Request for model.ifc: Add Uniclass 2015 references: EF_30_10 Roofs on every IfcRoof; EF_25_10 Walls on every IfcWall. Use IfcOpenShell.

First a look at what the model holds.

```python
import ifcopenshell

model = ifcopenshell.open("model.ifc")
print(model.schema)
print("classifications:", [c.Name for c in model.by_type("IfcClassification")])
for ifc_class in ("IfcDoor", "IfcRoof", "IfcStair", "IfcWall", "IfcWindow"):
    print(ifc_class, len(model.by_type(ifc_class)))
```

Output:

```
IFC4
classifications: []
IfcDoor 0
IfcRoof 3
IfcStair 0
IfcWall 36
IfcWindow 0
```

```python
import ifcopenshell
import ifcopenshell.api.classification

model = ifcopenshell.open("model.ifc")

system = ifcopenshell.api.classification.add_classification(model, classification="Uniclass 2015")

codes = {
    "IfcRoof": ("EF_30_10", "Roofs"),
    "IfcWall": ("EF_25_10", "Walls"),
}
for ifc_class, (code, name) in codes.items():
    products = model.by_type(ifc_class)
    ifcopenshell.api.classification.add_reference(
        model, products=products, classification=system, identification=code, name=name
    )
    print(code, len(products))

model.write("model_rev.ifc")
```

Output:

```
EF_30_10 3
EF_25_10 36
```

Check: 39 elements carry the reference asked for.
